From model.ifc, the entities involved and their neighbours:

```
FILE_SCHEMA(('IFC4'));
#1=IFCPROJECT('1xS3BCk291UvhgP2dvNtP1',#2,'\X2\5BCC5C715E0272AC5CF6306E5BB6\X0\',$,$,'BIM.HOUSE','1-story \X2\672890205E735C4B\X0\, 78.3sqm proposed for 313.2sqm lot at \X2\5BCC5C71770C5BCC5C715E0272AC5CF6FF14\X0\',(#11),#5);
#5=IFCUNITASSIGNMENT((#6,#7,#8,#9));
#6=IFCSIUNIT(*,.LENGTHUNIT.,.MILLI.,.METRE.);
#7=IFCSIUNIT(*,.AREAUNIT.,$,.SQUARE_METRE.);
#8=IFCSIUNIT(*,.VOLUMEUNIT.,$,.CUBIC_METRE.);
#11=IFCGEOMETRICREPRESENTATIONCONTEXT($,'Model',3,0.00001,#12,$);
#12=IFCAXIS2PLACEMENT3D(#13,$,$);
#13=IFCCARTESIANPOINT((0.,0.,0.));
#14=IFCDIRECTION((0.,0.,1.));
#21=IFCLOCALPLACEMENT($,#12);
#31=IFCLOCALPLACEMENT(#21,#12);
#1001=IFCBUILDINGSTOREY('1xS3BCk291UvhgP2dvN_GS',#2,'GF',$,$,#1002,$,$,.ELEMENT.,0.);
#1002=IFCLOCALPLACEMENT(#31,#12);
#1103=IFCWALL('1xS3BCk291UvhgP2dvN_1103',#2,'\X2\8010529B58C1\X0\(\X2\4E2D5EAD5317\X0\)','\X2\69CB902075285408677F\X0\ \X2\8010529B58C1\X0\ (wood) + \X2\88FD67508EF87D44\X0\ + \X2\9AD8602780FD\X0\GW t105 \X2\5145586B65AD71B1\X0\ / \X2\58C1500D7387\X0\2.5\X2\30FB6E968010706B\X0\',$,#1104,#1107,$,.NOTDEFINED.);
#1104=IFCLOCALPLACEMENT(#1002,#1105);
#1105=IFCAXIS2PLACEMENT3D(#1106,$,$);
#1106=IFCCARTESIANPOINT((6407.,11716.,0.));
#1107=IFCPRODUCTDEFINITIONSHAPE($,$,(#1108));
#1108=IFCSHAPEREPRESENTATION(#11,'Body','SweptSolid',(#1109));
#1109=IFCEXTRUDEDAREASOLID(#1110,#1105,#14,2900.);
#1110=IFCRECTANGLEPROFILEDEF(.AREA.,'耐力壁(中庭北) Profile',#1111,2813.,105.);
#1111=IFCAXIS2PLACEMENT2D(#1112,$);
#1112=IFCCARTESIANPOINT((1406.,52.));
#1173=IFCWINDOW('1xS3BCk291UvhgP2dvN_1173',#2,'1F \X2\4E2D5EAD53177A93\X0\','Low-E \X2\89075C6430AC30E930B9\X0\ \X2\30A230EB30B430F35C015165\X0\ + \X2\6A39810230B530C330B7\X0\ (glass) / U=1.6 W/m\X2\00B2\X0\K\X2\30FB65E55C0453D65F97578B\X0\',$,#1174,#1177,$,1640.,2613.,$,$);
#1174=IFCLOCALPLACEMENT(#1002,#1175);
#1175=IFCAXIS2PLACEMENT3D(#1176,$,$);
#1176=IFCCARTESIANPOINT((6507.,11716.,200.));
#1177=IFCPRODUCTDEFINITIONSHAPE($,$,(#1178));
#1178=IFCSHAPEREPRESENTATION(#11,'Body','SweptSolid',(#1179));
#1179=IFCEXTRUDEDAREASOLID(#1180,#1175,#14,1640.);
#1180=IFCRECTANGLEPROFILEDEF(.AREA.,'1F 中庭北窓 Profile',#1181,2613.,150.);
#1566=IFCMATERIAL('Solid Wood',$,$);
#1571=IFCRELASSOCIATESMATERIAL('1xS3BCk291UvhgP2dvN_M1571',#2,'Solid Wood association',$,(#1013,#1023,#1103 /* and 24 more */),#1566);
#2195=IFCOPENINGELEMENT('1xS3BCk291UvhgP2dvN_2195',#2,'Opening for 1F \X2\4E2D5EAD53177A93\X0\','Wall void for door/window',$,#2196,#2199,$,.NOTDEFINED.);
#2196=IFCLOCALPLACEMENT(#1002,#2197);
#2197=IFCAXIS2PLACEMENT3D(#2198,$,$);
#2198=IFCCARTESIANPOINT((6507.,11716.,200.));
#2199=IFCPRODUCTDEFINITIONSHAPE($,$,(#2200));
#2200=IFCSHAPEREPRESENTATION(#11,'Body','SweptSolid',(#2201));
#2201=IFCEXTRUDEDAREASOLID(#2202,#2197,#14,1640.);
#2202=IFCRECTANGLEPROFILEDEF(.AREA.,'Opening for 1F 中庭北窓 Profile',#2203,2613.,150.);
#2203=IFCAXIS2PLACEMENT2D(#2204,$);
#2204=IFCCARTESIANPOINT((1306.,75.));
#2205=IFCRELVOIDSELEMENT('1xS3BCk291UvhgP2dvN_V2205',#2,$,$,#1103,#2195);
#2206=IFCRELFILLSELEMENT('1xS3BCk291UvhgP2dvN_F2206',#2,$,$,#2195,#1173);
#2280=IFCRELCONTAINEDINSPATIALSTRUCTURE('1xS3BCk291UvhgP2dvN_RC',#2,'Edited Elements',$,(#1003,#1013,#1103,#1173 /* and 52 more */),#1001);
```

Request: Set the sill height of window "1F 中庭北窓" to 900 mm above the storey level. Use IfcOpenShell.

```python
import numpy as np
import ifcopenshell
import ifcopenshell.api.geometry
import ifcopenshell.geom
import ifcopenshell.util.element
import ifcopenshell.util.placement
import ifcopenshell.util.shape
import ifcopenshell.util.unit

model = ifcopenshell.open("model.ifc")
unit_scale = ifcopenshell.util.unit.calculate_unit_scale(model)

window = model.by_guid("1xS3BCk291UvhgP2dvN_1173")
opening = window.FillsVoids[0].RelatingOpeningElement
storey = ifcopenshell.util.element.get_container(window, ifc_class="IfcBuildingStorey")
level = ifcopenshell.util.placement.get_local_placement(storey.ObjectPlacement)[2, 3]

# The opening's origin need not be at the sill, so measure its lowest point.
shape = ifcopenshell.geom.create_shape(ifcopenshell.geom.settings(), opening)
bottom = ifcopenshell.util.shape.get_shape_bottom_elevation(shape, shape.geometry) / unit_scale
dz = level + 0.9 / unit_scale - bottom

shift = np.array([0.0, 0.0, dz])
# The window is not placed relative to its opening, so move both.
for product in (opening, window):
    matrix = ifcopenshell.util.placement.get_local_placement(product.ObjectPlacement)
    matrix[:3, 3] += shift
    ifcopenshell.api.geometry.edit_object_placement(model, product=product, matrix=matrix, is_si=False)

print(f"moved by {dz * unit_scale:+.3f} m")

model.write("model-out.ifc")
```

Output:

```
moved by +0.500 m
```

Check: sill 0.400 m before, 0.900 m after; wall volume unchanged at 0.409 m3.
